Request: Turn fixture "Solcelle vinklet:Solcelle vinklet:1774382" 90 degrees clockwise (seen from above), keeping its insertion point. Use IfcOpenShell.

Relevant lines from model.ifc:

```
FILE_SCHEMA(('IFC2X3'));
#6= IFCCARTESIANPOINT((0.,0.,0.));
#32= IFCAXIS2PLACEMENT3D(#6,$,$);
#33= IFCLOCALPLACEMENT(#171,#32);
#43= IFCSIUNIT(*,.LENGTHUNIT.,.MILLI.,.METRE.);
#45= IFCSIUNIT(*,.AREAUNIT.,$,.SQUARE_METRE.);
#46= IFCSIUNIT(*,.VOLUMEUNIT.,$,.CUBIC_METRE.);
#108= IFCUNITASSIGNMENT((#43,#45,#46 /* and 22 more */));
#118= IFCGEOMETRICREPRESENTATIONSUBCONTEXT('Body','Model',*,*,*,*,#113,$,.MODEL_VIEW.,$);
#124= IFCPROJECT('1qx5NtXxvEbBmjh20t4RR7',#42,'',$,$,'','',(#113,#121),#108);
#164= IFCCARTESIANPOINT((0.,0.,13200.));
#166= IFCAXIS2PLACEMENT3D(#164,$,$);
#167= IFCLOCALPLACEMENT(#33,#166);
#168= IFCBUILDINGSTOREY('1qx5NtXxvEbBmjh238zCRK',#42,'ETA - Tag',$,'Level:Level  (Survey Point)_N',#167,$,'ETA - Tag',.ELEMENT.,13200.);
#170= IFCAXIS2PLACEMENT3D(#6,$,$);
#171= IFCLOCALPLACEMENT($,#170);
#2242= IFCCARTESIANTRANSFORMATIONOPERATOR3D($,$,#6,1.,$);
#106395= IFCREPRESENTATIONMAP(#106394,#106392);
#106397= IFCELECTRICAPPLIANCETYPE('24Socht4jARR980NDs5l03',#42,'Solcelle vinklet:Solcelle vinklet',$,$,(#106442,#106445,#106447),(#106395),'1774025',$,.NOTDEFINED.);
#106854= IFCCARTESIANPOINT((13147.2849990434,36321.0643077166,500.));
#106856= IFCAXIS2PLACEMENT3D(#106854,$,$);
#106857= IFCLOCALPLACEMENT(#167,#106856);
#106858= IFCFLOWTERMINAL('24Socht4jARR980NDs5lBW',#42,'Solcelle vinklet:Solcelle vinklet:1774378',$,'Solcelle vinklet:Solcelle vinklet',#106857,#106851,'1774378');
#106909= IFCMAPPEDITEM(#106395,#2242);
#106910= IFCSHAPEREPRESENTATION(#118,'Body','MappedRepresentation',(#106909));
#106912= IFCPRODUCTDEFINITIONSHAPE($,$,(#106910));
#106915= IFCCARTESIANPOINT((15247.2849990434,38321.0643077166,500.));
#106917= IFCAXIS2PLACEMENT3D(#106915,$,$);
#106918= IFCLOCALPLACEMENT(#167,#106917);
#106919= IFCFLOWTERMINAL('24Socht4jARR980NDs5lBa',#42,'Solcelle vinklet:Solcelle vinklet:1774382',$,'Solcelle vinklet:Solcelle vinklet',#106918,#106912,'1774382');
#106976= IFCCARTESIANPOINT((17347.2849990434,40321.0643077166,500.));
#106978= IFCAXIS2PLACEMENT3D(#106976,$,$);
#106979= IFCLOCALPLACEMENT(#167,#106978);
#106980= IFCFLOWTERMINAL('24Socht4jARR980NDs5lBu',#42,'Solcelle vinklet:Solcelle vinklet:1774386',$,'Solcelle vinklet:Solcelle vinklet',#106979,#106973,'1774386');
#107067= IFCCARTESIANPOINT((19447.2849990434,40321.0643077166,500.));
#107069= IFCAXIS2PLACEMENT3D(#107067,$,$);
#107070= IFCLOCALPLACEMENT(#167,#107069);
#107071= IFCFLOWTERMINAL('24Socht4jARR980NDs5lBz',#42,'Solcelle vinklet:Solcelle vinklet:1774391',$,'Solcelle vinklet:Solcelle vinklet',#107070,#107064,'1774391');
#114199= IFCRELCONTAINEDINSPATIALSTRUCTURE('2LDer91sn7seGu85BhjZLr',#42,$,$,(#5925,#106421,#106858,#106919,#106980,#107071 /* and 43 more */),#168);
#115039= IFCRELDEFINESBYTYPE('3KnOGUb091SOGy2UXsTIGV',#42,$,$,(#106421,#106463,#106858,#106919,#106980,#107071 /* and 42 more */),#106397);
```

```python
import ifcopenshell
import ifcopenshell.api.geometry
import ifcopenshell.util.placement

model = ifcopenshell.open("model.ifc")

item = model.by_id(106919)
matrix = ifcopenshell.util.placement.get_local_placement(item.ObjectPlacement)
matrix = matrix @ ifcopenshell.util.placement.rotation(-90, "Z")
ifcopenshell.api.geometry.edit_object_placement(model, product=item, matrix=matrix, is_si=False)

print(ifcopenshell.util.placement.get_local_placement(item.ObjectPlacement).round(3) + 0.0)

model.write("model_edited.ifc")
```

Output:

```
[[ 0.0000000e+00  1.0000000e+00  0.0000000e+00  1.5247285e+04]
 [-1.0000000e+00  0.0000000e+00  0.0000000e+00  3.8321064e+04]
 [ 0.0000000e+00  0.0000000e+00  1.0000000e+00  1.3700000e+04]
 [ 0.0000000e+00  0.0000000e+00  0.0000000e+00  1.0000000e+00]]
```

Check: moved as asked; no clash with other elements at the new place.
